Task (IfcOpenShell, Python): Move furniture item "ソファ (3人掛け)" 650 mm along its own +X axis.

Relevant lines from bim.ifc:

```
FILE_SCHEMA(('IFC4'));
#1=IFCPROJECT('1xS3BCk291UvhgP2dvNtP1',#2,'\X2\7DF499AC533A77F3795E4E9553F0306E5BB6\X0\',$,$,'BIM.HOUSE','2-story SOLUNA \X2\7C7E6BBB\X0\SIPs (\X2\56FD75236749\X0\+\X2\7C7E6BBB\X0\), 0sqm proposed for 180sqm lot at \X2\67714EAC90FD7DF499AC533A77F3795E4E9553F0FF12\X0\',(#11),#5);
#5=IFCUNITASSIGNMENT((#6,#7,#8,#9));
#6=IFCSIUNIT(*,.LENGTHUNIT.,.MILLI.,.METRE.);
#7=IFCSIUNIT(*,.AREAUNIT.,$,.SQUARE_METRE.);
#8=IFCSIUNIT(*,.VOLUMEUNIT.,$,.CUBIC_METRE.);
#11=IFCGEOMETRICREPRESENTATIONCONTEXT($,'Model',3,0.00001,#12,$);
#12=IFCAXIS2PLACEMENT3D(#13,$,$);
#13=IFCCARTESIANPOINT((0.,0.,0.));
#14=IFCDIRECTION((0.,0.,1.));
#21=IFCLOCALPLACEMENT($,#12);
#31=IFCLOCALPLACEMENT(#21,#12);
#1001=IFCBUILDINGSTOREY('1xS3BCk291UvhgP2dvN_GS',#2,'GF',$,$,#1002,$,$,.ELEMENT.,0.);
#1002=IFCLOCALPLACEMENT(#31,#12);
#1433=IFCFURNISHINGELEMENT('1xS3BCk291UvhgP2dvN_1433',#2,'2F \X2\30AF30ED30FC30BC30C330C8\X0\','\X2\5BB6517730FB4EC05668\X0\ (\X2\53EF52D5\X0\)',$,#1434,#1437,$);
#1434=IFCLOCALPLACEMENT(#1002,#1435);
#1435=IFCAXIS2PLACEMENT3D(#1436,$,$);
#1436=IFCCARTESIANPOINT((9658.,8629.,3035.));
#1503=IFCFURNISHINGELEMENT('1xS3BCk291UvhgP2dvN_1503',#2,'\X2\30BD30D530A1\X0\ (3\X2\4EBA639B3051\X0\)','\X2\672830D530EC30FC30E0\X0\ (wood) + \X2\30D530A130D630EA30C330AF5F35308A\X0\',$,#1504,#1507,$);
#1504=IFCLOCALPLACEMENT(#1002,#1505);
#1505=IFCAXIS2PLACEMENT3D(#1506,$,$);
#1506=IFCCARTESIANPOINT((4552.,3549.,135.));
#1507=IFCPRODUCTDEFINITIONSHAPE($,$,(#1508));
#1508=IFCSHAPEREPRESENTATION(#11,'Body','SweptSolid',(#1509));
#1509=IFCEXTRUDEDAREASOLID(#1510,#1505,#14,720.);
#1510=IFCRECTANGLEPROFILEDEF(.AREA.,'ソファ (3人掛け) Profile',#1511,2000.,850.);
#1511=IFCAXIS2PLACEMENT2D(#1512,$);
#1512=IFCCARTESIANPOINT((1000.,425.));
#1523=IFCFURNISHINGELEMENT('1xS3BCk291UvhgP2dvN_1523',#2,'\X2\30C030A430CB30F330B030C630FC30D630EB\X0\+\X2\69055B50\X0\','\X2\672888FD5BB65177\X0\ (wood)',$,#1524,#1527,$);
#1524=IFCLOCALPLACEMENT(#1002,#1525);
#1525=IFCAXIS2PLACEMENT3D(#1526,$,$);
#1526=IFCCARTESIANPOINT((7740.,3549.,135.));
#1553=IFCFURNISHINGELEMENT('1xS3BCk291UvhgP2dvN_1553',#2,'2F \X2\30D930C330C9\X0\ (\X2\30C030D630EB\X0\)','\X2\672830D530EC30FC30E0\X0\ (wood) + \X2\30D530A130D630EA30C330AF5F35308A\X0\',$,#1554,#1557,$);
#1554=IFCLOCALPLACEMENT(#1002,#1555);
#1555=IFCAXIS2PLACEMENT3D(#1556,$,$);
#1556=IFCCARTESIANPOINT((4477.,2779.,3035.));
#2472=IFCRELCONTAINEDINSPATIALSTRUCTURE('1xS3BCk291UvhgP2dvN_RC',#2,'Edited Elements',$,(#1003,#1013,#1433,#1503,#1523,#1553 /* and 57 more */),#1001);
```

```python
import ifcopenshell
import ifcopenshell.api.geometry
import ifcopenshell.util.placement
import ifcopenshell.util.unit

model = ifcopenshell.open("bim.ifc")
unit_scale = ifcopenshell.util.unit.calculate_unit_scale(model)

item = model.by_id(1503)
matrix = ifcopenshell.util.placement.get_local_placement(item.ObjectPlacement)
matrix[:3, 3] += matrix[:3, 0] * 0.65 / unit_scale
ifcopenshell.api.geometry.edit_object_placement(model, product=item, matrix=matrix, is_si=False)

print(ifcopenshell.util.placement.get_local_placement(item.ObjectPlacement).round(3) + 0.0)

model.write("bim_edited.ifc")
```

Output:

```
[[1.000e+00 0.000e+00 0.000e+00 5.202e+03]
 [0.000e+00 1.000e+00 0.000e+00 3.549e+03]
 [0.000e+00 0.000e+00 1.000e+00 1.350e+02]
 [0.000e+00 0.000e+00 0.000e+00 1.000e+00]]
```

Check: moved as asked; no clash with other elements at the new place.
